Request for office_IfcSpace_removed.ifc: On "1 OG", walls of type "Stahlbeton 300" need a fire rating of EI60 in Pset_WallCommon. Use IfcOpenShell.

First a look at what the model holds.

```python
import ifcopenshell
import ifcopenshell.util.element

model = ifcopenshell.open("office_IfcSpace_removed.ifc")
print(model.schema)
storey = next(s for s in model.by_type("IfcBuildingStorey") if s.Name == "1 OG")
walls = [e for e in ifcopenshell.util.element.get_decomposition(storey) if e.is_a("IfcWall")]
seen = {}
for e in walls:
    element_type = ifcopenshell.util.element.get_type(e)
    key = (element_type.Name if element_type != e and element_type else None, ifcopenshell.util.element.get_pset(e, "Pset_WallCommon", "FireRating"))
    seen[key] = seen.get(key, 0) + 1
for (name, value), count in sorted(seen.items(), key=str):
    print(count, "x", name, "|", value)
```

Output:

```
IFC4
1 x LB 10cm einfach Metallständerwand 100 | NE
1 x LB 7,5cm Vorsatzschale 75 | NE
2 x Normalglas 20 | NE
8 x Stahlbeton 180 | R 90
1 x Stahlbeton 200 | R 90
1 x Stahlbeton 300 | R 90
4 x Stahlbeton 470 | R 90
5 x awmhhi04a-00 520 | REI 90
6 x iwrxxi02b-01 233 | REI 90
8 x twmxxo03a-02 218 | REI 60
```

```python
import ifcopenshell
import ifcopenshell.api.pset
import ifcopenshell.util.element

model = ifcopenshell.open("office_IfcSpace_removed.ifc")

storey = next(s for s in model.by_type("IfcBuildingStorey") if s.Name == "1 OG")
walls = [e for e in ifcopenshell.util.element.get_decomposition(storey) if e.is_a("IfcWall")]

count = 0
for e in walls:
    element_type = ifcopenshell.util.element.get_type(e)
    if element_type in (None, e) or element_type.Name != "Stahlbeton 300":
        continue
    # add_pset returns the element's existing set when there is one.
    pset = ifcopenshell.api.pset.add_pset(model, product=e, name="Pset_WallCommon")
    ifcopenshell.api.pset.edit_pset(model, pset=pset, properties={"FireRating": "EI60"})
    count += 1

print(count, "walls updated")

model.write("office_IfcSpace_removed_v2.ifc")
```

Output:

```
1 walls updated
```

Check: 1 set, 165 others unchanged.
